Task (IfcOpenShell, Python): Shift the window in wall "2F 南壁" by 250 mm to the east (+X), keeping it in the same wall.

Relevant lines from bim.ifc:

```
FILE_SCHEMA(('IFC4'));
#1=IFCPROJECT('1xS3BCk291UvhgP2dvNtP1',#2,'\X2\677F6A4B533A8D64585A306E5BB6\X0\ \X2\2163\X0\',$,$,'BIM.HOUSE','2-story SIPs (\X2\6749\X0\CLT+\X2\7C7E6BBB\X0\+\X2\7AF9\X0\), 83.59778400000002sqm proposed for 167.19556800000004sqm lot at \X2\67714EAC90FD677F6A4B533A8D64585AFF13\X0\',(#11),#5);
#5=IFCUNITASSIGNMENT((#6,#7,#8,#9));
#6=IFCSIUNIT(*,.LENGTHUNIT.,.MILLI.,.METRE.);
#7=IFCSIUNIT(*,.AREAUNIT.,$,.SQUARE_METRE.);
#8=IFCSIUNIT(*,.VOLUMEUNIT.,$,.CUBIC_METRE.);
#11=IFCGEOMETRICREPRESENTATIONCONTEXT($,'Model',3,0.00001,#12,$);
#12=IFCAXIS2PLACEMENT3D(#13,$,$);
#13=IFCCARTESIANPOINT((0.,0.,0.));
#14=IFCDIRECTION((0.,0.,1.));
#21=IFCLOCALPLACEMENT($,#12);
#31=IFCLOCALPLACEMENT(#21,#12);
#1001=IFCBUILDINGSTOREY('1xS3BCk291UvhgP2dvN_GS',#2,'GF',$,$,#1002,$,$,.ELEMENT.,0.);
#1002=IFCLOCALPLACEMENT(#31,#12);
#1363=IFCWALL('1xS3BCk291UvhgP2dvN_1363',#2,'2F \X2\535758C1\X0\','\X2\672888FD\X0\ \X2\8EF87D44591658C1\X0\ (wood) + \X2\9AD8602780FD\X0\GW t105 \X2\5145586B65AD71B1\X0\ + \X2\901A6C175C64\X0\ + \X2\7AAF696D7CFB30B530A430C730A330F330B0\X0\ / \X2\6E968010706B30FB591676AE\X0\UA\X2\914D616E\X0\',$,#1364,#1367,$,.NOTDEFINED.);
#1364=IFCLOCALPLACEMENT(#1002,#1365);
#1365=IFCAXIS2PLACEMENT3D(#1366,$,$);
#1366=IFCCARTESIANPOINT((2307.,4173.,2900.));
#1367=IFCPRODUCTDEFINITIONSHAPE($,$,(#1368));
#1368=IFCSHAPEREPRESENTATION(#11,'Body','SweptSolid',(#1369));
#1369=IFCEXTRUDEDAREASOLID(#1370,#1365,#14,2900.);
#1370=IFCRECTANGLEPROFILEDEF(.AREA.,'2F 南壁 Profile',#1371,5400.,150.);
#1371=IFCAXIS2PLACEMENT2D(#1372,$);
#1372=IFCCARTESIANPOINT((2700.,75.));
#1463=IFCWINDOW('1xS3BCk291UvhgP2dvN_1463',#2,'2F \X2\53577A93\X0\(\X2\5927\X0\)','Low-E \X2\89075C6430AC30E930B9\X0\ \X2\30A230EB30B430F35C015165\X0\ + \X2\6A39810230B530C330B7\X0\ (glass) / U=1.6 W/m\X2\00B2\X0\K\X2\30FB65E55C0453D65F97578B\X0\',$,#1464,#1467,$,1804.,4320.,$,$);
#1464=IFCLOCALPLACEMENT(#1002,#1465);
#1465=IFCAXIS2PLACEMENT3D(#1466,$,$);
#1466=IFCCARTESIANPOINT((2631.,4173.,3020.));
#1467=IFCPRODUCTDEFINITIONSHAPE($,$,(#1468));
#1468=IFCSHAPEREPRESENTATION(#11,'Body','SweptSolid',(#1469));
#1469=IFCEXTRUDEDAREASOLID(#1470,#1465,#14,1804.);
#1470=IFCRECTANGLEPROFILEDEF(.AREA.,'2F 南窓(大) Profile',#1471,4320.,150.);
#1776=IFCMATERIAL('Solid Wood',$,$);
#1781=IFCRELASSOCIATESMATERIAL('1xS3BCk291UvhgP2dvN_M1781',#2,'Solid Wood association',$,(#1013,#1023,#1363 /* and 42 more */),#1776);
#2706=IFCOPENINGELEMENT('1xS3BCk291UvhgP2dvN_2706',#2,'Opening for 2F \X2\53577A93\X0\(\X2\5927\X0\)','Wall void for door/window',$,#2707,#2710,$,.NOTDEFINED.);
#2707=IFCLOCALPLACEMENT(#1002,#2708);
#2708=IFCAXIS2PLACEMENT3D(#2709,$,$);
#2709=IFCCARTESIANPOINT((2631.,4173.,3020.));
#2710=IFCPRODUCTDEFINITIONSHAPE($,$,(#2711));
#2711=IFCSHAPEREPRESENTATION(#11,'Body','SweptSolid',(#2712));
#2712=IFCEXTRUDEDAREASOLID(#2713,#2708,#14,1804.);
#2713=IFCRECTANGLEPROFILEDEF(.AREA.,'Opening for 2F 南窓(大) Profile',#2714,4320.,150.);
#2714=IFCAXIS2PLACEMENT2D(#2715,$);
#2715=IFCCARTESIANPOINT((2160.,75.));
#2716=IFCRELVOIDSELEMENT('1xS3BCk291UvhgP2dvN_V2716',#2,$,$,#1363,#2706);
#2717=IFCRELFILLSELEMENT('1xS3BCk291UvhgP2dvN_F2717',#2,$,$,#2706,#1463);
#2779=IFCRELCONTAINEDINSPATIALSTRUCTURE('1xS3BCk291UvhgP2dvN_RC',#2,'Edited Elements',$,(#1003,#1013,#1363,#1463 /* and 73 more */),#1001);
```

```python
import ifcopenshell
import ifcopenshell.api.geometry
import ifcopenshell.util.placement
import ifcopenshell.util.unit

model = ifcopenshell.open("bim.ifc")
unit_scale = ifcopenshell.util.unit.calculate_unit_scale(model)

window = model.by_id(1463)
opening = window.FillsVoids[0].RelatingOpeningElement
wall = opening.VoidsElements[0].RelatingBuildingElement

wall_matrix = ifcopenshell.util.placement.get_local_placement(wall.ObjectPlacement)
shift = wall_matrix[:3, 0] * 0.25 / unit_scale
before = ifcopenshell.util.placement.get_local_placement(window.ObjectPlacement)[:3, 3].copy()

# The window is not placed relative to its opening, so move both.
for product in (opening, window):
    matrix = ifcopenshell.util.placement.get_local_placement(product.ObjectPlacement)
    matrix[:3, 3] += shift
    ifcopenshell.api.geometry.edit_object_placement(model, product=product, matrix=matrix, is_si=False)

after = ifcopenshell.util.placement.get_local_placement(window.ObjectPlacement)[:3, 3]
print("window moved by", (after - before).round(3) + 0.0)

model.write("bim_updated.ifc")
```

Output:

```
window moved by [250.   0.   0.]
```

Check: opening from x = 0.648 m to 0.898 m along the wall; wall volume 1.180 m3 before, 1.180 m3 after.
